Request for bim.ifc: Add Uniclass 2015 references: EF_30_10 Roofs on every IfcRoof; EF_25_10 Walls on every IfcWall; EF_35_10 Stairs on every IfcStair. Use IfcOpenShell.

First a look at what the model holds.

```python
import ifcopenshell

model = ifcopenshell.open("bim.ifc")
print(model.schema)
print("classifications:", [c.Name for c in model.by_type("IfcClassification")])
for ifc_class in ("IfcDoor", "IfcRoof", "IfcStair", "IfcWall", "IfcWindow"):
    print(ifc_class, len(model.by_type(ifc_class)))
```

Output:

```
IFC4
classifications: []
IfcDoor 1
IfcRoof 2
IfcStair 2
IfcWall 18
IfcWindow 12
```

```python
import ifcopenshell
import ifcopenshell.api.classification

model = ifcopenshell.open("bim.ifc")

system = ifcopenshell.api.classification.add_classification(model, classification="Uniclass 2015")

codes = {
    "IfcRoof": ("EF_30_10", "Roofs"),
    "IfcWall": ("EF_25_10", "Walls"),
    "IfcStair": ("EF_35_10", "Stairs"),
}
for ifc_class, (code, name) in codes.items():
    products = model.by_type(ifc_class)
    ifcopenshell.api.classification.add_reference(
        model, products=products, classification=system, identification=code, name=name
    )
    print(code, len(products))

model.write("bim_updated.ifc")
```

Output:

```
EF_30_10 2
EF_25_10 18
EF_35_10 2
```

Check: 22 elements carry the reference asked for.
